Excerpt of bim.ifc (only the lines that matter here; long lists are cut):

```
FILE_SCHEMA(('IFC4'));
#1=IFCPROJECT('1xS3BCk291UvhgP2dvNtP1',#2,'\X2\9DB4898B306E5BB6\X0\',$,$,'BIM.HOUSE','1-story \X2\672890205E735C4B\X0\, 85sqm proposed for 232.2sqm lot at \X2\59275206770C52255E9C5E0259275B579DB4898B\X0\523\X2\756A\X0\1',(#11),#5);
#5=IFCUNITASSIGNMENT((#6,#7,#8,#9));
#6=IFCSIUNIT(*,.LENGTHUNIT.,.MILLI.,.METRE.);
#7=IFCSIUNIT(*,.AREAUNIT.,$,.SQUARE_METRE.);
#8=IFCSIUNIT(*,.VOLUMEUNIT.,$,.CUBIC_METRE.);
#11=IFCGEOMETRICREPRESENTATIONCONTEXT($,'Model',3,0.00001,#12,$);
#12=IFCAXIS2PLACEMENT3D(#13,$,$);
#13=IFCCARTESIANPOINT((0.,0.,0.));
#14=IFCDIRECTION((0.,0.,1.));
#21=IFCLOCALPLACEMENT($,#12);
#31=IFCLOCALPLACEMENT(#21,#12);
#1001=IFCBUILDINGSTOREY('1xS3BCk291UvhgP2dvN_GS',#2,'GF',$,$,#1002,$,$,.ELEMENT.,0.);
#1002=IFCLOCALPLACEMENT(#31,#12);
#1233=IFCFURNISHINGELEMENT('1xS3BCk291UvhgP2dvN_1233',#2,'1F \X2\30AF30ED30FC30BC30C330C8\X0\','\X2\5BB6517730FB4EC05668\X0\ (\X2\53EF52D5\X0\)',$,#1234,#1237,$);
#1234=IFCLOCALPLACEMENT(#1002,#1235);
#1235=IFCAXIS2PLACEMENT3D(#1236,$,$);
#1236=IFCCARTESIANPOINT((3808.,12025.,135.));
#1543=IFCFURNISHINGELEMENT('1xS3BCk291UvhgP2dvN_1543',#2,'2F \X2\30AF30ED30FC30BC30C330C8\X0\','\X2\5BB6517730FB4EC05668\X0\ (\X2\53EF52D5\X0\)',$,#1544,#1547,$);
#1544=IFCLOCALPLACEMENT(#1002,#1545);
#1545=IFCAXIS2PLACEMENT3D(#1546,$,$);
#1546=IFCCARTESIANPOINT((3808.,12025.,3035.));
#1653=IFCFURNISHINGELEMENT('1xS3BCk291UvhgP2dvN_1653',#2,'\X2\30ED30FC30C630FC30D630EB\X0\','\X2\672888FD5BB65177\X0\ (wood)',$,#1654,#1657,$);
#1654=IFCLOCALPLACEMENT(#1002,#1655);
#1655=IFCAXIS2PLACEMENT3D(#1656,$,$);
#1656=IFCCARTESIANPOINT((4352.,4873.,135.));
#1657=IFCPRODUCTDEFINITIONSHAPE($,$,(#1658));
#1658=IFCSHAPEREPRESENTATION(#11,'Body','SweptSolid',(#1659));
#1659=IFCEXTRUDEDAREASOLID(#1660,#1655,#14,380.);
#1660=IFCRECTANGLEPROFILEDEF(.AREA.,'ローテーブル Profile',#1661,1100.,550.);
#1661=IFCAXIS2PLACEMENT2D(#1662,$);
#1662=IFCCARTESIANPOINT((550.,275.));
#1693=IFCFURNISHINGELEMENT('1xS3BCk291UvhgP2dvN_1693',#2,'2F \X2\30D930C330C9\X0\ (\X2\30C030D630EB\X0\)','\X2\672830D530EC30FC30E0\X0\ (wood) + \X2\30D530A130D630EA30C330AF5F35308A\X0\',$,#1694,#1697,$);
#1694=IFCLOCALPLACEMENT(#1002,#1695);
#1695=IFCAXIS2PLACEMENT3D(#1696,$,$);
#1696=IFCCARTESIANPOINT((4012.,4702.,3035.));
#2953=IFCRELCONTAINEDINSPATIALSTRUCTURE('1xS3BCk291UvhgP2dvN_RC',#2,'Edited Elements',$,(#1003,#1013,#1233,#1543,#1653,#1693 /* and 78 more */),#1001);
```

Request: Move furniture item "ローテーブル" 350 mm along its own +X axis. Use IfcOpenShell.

```python
import ifcopenshell
import ifcopenshell.api.geometry
import ifcopenshell.util.placement

model = ifcopenshell.open("bim.ifc")

item = model.by_id(1653)
matrix = ifcopenshell.util.placement.get_local_placement(item.ObjectPlacement)
matrix[:3, 3] += matrix[:3, 0] * 350.0
ifcopenshell.api.geometry.edit_object_placement(model, product=item, matrix=matrix, is_si=False)

print(ifcopenshell.util.placement.get_local_placement(item.ObjectPlacement).round(3) + 0.0)

model.write("bim_edited.ifc")
```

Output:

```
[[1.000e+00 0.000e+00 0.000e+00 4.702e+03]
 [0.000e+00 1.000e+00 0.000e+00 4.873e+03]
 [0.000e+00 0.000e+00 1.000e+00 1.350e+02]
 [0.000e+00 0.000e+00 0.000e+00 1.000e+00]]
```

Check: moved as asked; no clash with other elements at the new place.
